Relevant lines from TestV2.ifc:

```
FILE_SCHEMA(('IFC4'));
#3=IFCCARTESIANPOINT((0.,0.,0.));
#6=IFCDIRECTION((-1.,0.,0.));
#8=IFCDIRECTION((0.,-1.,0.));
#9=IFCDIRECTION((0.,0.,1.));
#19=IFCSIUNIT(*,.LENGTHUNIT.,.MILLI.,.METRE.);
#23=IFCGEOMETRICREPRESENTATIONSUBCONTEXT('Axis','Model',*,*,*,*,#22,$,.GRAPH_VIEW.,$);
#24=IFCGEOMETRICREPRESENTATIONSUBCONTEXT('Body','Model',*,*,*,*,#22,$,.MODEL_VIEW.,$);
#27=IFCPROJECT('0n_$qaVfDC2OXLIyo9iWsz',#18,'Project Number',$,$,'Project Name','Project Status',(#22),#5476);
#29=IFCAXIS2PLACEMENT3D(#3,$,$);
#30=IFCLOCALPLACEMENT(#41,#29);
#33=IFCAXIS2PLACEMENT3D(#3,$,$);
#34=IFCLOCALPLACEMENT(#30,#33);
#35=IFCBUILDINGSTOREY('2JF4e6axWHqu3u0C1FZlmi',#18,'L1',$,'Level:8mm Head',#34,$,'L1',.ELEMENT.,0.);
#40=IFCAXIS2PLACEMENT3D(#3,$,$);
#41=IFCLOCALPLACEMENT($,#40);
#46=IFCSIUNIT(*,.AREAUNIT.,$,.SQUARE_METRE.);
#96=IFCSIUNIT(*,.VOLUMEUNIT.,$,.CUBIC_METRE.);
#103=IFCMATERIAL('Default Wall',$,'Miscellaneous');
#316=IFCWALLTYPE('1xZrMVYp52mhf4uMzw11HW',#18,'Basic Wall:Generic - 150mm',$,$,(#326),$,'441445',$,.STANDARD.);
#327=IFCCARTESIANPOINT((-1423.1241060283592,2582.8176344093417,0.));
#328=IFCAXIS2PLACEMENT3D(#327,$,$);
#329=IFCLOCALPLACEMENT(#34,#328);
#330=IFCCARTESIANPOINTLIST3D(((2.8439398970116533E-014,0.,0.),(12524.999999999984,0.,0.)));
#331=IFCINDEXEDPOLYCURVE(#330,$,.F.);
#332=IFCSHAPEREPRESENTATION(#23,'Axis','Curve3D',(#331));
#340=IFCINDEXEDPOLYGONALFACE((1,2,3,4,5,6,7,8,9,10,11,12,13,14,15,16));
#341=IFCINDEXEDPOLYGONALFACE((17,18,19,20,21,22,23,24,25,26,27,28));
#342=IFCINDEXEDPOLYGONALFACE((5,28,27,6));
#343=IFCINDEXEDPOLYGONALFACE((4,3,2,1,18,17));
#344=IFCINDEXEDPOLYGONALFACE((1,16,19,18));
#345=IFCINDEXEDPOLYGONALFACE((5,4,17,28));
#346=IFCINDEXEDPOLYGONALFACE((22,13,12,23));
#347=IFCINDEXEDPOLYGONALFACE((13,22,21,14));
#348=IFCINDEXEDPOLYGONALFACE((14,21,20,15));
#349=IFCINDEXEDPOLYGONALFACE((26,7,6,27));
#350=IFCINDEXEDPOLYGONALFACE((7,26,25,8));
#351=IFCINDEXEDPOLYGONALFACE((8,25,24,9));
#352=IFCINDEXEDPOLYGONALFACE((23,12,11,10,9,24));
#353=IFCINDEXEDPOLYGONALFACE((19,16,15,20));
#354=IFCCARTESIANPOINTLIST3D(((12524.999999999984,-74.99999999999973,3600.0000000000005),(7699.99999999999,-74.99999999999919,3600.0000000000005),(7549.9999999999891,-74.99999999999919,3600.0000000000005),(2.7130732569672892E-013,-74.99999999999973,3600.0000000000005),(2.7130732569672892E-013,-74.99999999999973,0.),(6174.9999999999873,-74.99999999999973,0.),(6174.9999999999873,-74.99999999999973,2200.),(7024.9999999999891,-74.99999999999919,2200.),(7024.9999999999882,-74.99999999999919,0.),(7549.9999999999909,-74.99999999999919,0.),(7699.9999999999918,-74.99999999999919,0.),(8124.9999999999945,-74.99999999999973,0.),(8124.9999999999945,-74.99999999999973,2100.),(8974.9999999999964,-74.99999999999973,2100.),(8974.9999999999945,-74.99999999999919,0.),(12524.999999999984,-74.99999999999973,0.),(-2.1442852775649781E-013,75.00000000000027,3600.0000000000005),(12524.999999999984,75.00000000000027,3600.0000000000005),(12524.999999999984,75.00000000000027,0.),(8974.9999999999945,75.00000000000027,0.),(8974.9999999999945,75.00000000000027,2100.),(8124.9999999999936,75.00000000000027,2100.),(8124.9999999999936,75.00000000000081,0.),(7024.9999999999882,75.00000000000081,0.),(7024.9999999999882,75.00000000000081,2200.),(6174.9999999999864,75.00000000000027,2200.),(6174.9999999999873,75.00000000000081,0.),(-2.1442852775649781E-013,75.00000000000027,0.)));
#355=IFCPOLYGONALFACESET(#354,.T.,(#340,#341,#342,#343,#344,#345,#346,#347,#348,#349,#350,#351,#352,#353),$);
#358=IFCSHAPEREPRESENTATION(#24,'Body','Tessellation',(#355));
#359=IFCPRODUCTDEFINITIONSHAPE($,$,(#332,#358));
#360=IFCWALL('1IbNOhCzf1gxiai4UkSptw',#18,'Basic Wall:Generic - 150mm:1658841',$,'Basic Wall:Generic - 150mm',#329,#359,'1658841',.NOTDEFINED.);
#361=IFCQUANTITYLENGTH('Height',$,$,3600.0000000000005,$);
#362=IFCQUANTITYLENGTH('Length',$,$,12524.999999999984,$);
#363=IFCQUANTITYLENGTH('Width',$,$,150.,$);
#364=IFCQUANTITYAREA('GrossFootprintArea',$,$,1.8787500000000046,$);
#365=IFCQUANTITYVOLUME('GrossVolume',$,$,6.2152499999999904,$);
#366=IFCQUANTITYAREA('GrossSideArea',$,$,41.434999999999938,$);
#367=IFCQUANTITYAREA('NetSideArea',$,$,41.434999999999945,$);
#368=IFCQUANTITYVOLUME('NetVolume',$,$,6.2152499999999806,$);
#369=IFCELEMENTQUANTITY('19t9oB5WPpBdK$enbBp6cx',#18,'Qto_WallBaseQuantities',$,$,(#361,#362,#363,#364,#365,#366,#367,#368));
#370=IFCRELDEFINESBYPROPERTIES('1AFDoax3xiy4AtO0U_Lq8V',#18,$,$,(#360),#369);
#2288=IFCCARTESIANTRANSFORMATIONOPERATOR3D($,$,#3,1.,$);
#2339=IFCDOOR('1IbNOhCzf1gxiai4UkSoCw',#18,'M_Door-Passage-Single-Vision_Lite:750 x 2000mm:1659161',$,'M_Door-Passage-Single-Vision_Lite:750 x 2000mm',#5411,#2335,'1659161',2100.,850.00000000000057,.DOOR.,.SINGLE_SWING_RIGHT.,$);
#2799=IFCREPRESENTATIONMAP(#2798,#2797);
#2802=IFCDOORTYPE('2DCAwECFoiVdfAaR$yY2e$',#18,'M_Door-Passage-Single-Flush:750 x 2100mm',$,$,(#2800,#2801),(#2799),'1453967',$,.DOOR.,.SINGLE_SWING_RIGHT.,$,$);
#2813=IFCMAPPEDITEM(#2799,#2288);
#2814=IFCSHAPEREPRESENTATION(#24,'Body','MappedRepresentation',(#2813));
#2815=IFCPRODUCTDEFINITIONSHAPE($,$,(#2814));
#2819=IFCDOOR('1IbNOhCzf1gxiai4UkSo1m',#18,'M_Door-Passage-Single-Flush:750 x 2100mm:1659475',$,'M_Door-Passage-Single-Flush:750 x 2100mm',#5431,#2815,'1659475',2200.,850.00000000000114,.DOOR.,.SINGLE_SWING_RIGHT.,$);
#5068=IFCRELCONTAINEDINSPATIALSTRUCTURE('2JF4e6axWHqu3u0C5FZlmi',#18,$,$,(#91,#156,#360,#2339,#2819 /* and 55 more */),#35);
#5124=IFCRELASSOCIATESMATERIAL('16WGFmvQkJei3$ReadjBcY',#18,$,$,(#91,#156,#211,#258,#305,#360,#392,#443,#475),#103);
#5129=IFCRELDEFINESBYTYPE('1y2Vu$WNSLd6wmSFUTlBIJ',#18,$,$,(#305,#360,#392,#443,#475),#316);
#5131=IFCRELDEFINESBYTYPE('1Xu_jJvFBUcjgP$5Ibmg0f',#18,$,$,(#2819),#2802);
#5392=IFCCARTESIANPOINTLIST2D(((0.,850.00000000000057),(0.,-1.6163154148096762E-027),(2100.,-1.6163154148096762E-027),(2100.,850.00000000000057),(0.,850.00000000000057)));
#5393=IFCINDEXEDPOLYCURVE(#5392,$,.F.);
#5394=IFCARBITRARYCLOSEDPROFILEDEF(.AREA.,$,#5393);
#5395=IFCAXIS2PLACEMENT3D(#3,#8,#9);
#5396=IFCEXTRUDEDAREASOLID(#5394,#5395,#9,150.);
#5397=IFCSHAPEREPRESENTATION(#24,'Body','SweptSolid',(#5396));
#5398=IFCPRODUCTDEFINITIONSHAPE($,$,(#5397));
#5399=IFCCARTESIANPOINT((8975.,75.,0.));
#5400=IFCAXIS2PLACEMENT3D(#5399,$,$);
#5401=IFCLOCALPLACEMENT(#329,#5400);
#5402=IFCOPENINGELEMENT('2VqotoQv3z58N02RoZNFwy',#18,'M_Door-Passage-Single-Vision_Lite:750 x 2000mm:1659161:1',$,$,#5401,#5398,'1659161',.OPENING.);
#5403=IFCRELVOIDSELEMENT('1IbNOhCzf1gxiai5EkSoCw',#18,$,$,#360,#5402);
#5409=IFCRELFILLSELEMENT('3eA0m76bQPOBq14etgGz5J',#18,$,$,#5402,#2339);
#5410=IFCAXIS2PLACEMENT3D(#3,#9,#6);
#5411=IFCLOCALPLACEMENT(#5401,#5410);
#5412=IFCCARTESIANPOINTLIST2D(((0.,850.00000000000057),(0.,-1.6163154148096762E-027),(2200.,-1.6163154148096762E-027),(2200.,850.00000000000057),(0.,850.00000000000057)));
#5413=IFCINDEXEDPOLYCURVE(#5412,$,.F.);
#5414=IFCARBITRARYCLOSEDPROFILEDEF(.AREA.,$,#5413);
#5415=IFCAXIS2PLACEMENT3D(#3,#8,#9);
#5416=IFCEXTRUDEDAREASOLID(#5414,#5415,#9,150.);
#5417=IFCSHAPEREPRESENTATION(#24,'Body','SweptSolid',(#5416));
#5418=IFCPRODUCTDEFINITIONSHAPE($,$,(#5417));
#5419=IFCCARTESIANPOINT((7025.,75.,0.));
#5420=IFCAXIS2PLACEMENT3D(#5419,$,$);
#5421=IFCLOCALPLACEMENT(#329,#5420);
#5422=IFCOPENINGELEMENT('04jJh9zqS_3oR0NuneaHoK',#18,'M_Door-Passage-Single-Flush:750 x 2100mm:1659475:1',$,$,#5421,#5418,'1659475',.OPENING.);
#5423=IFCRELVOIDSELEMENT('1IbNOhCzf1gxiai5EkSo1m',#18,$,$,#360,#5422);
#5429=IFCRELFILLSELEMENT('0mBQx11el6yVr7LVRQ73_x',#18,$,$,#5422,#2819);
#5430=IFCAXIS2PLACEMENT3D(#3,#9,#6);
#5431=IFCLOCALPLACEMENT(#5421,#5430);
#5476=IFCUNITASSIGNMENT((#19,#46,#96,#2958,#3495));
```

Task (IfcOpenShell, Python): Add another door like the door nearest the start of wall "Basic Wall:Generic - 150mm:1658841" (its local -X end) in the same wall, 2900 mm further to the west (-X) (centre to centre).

```python
import ifcopenshell
import ifcopenshell.api.feature
import ifcopenshell.api.geometry
import ifcopenshell.api.pset
import ifcopenshell.api.root
import ifcopenshell.geom
import ifcopenshell.util.element
import ifcopenshell.util.placement
import ifcopenshell.util.shape
import ifcopenshell.util.unit

model = ifcopenshell.open("TestV2.ifc")
area_scale = ifcopenshell.util.unit.calculate_unit_scale(model, "AREAUNIT")
volume_scale = ifcopenshell.util.unit.calculate_unit_scale(model, "VOLUMEUNIT")
settings = ifcopenshell.geom.settings()


def volume(element):
    """Net volume in cubic metres, openings subtracted."""
    shape = ifcopenshell.geom.create_shape(settings, element)
    return ifcopenshell.util.shape.get_volume(shape.geometry)


def reuse_history(source, copy):
    """copy_class also copies each property set's owner history, people and application; keep the originals."""
    for rel in copy.IsDefinedBy:
        if rel.is_a("IfcRelDefinesByProperties") and (history := rel.RelatingPropertyDefinition.OwnerHistory):
            rel.RelatingPropertyDefinition.OwnerHistory = source.OwnerHistory
            ifcopenshell.util.element.remove_deep2(model, history)


door = model.by_guid("1IbNOhCzf1gxiai4UkSo1m")
opening = door.FillsVoids[0].RelatingOpeningElement
wall = opening.VoidsElements[0].RelatingBuildingElement
before = volume(wall)
shift = ifcopenshell.util.placement.get_local_placement(wall.ObjectPlacement)[:3, 0] * -2900.0

# copy_class copies the void relationship, type, container and properties, but no geometry.
new_opening = ifcopenshell.api.root.copy_class(model, product=opening)
new_opening.Representation = ifcopenshell.util.element.copy_deep(
    model, opening.Representation, exclude=["IfcGeometricRepresentationContext", "IfcRepresentationMap"]
)
new_opening.Name = "M_Door-Passage-Single-Flush:750 x 2100mm"
new_opening.Tag = None
reuse_history(opening, new_opening)
new_door = ifcopenshell.api.root.copy_class(model, product=door)
new_door.Representation = ifcopenshell.util.element.copy_deep(
    model, door.Representation, exclude=["IfcGeometricRepresentationContext", "IfcRepresentationMap"]
)
new_door.Name = "M_Door-Passage-Single-Flush:750 x 2100mm"
new_door.Tag = None
reuse_history(door, new_door)
ifcopenshell.api.feature.add_filling(model, opening=new_opening, element=new_door)

for old, new in ((opening, new_opening), (door, new_door)):
    matrix = ifcopenshell.util.placement.get_local_placement(old.ObjectPlacement)
    matrix[:3, 3] += shift
    ifcopenshell.api.geometry.edit_object_placement(model, product=new, matrix=matrix, is_si=False)

after = volume(wall)
thickness = 0.15  # wall thickness in metres

# Update the wall's stored quantities.
qto = model.by_id(ifcopenshell.util.element.get_pset(wall, "Qto_WallBaseQuantities", should_inherit=False)["id"])
ifcopenshell.api.pset.edit_qto(model, qto=qto, properties={
    "NetSideArea": after / thickness / area_scale,
    "NetVolume": after / volume_scale,
})

print(f"wall volume {before:.3f} -> {after:.3f} m3")

model.write("TestV2_edited.ifc")
```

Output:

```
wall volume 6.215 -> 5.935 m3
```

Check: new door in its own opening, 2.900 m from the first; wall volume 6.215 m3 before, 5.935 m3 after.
